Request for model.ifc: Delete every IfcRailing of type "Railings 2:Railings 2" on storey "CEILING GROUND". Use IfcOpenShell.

First a look at what the model holds.

```python
import ifcopenshell
import ifcopenshell.util.element

model = ifcopenshell.open("model.ifc")
print(model.schema)
storey = next(s for s in model.by_type("IfcBuildingStorey") if s.Name == "CEILING GROUND")
railings = [e for e in ifcopenshell.util.element.get_decomposition(storey) if e.is_a("IfcRailing")]
seen = {}
for e in railings:
    element_type = ifcopenshell.util.element.get_type(e)
    name = element_type.Name if element_type not in (None, e) else None
    seen[name] = seen.get(name, 0) + 1
for name, count in sorted(seen.items(), key=str):
    print(count, "x", name)
```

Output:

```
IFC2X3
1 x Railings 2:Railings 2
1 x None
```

```python
import ifcopenshell
import ifcopenshell.api.root
import ifcopenshell.util.element

model = ifcopenshell.open("model.ifc")

storey = next(s for s in model.by_type("IfcBuildingStorey") if s.Name == "CEILING GROUND")
railings = [e for e in ifcopenshell.util.element.get_decomposition(storey) if e.is_a("IfcRailing")]
targets = [e for e in railings if (t := ifcopenshell.util.element.get_type(e)) not in (None, e) and t.Name == "Railings 2:Railings 2"]

for e in targets:
    ifcopenshell.api.root.remove_product(model, product=e)
print(len(targets), "removed")

model.write("model-out.ifc")
```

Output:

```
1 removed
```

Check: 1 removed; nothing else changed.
